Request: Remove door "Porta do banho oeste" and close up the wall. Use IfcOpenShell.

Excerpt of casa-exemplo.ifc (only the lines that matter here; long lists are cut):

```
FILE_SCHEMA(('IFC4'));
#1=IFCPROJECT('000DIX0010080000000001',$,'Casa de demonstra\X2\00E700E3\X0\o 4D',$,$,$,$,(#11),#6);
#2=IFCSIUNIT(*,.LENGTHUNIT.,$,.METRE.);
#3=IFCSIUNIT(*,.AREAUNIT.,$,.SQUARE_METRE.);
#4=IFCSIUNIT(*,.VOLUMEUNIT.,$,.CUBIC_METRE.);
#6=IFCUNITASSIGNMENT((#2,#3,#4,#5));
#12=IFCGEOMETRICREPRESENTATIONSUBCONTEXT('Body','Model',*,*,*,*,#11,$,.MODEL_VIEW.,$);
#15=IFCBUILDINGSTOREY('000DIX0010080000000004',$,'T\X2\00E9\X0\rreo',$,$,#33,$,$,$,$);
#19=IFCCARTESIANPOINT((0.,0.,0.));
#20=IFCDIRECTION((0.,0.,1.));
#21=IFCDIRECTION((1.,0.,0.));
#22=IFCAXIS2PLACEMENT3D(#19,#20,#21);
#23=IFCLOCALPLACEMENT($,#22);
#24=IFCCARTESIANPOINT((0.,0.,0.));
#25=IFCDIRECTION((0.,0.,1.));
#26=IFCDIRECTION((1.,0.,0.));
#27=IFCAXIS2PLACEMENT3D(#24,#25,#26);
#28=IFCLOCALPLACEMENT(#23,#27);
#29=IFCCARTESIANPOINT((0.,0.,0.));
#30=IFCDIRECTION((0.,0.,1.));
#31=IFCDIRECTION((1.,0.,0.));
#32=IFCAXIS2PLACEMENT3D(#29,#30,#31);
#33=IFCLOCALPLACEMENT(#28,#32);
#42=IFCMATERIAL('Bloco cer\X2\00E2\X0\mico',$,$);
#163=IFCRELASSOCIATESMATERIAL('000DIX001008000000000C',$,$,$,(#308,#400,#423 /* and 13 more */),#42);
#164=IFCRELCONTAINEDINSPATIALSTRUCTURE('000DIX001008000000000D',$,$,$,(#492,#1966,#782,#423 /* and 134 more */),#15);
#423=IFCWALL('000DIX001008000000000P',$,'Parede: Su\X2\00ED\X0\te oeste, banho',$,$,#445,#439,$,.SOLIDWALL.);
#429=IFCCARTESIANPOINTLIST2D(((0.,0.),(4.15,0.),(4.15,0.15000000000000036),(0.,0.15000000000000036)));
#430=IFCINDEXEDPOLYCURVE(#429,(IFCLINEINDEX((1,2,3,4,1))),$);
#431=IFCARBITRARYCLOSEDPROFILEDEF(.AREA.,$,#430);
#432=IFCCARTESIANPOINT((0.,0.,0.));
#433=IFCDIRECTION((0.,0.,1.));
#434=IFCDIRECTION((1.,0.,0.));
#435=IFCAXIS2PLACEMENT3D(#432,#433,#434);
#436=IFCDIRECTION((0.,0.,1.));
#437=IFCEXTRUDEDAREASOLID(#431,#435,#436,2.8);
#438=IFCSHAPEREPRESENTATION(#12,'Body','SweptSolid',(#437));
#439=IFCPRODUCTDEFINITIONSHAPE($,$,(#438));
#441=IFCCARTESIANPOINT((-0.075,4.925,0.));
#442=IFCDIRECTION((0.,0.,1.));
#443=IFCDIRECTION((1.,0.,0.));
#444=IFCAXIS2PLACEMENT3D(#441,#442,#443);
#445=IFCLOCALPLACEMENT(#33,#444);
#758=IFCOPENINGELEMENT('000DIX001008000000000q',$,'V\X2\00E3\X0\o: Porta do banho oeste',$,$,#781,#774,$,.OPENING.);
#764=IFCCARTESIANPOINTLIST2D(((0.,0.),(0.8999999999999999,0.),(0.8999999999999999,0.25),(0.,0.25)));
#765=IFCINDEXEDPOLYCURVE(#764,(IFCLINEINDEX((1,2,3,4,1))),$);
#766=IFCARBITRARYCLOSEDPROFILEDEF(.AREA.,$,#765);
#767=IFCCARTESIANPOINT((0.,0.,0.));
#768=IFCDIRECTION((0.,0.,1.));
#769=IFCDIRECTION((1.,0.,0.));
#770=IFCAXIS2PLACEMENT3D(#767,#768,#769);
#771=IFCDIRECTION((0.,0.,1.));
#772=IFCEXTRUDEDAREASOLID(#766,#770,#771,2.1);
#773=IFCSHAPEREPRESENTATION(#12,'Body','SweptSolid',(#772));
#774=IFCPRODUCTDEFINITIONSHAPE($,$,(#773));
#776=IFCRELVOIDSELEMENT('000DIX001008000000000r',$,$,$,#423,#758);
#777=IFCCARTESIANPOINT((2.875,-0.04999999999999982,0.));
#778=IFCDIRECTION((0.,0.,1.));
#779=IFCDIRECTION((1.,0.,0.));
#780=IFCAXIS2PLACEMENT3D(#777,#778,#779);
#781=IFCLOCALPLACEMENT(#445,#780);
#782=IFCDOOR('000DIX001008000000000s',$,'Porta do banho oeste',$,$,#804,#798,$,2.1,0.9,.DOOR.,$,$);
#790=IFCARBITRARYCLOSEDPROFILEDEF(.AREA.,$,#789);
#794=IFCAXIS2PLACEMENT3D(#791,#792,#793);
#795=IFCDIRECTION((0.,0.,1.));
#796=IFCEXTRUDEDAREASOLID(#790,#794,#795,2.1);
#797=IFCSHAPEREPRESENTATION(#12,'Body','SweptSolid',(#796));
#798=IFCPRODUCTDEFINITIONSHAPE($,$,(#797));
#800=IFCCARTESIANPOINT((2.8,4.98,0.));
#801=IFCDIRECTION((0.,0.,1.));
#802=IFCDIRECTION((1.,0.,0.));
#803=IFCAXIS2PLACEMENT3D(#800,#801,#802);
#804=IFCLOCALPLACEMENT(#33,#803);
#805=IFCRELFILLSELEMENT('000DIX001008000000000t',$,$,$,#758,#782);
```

```python
import ifcopenshell
import ifcopenshell.api.feature
import ifcopenshell.api.root
import ifcopenshell.geom
import ifcopenshell.util.shape

model = ifcopenshell.open("casa-exemplo.ifc")
settings = ifcopenshell.geom.settings()


def volume(element):
    """Net volume in cubic metres, openings subtracted."""
    shape = ifcopenshell.geom.create_shape(settings, element)
    return ifcopenshell.util.shape.get_volume(shape.geometry)


door = model.by_id(782)
opening = door.FillsVoids[0].RelatingOpeningElement
wall = opening.VoidsElements[0].RelatingBuildingElement
before = volume(wall)

ifcopenshell.api.root.remove_product(model, product=door)
ifcopenshell.api.feature.remove_feature(model, feature=opening)

after = volume(wall)

print(f"wall volume {before:.3f} -> {after:.3f} m3")

model.write("casa-exemplo_v2.ifc")
```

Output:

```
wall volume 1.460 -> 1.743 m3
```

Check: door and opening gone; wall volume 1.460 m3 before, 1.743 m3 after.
